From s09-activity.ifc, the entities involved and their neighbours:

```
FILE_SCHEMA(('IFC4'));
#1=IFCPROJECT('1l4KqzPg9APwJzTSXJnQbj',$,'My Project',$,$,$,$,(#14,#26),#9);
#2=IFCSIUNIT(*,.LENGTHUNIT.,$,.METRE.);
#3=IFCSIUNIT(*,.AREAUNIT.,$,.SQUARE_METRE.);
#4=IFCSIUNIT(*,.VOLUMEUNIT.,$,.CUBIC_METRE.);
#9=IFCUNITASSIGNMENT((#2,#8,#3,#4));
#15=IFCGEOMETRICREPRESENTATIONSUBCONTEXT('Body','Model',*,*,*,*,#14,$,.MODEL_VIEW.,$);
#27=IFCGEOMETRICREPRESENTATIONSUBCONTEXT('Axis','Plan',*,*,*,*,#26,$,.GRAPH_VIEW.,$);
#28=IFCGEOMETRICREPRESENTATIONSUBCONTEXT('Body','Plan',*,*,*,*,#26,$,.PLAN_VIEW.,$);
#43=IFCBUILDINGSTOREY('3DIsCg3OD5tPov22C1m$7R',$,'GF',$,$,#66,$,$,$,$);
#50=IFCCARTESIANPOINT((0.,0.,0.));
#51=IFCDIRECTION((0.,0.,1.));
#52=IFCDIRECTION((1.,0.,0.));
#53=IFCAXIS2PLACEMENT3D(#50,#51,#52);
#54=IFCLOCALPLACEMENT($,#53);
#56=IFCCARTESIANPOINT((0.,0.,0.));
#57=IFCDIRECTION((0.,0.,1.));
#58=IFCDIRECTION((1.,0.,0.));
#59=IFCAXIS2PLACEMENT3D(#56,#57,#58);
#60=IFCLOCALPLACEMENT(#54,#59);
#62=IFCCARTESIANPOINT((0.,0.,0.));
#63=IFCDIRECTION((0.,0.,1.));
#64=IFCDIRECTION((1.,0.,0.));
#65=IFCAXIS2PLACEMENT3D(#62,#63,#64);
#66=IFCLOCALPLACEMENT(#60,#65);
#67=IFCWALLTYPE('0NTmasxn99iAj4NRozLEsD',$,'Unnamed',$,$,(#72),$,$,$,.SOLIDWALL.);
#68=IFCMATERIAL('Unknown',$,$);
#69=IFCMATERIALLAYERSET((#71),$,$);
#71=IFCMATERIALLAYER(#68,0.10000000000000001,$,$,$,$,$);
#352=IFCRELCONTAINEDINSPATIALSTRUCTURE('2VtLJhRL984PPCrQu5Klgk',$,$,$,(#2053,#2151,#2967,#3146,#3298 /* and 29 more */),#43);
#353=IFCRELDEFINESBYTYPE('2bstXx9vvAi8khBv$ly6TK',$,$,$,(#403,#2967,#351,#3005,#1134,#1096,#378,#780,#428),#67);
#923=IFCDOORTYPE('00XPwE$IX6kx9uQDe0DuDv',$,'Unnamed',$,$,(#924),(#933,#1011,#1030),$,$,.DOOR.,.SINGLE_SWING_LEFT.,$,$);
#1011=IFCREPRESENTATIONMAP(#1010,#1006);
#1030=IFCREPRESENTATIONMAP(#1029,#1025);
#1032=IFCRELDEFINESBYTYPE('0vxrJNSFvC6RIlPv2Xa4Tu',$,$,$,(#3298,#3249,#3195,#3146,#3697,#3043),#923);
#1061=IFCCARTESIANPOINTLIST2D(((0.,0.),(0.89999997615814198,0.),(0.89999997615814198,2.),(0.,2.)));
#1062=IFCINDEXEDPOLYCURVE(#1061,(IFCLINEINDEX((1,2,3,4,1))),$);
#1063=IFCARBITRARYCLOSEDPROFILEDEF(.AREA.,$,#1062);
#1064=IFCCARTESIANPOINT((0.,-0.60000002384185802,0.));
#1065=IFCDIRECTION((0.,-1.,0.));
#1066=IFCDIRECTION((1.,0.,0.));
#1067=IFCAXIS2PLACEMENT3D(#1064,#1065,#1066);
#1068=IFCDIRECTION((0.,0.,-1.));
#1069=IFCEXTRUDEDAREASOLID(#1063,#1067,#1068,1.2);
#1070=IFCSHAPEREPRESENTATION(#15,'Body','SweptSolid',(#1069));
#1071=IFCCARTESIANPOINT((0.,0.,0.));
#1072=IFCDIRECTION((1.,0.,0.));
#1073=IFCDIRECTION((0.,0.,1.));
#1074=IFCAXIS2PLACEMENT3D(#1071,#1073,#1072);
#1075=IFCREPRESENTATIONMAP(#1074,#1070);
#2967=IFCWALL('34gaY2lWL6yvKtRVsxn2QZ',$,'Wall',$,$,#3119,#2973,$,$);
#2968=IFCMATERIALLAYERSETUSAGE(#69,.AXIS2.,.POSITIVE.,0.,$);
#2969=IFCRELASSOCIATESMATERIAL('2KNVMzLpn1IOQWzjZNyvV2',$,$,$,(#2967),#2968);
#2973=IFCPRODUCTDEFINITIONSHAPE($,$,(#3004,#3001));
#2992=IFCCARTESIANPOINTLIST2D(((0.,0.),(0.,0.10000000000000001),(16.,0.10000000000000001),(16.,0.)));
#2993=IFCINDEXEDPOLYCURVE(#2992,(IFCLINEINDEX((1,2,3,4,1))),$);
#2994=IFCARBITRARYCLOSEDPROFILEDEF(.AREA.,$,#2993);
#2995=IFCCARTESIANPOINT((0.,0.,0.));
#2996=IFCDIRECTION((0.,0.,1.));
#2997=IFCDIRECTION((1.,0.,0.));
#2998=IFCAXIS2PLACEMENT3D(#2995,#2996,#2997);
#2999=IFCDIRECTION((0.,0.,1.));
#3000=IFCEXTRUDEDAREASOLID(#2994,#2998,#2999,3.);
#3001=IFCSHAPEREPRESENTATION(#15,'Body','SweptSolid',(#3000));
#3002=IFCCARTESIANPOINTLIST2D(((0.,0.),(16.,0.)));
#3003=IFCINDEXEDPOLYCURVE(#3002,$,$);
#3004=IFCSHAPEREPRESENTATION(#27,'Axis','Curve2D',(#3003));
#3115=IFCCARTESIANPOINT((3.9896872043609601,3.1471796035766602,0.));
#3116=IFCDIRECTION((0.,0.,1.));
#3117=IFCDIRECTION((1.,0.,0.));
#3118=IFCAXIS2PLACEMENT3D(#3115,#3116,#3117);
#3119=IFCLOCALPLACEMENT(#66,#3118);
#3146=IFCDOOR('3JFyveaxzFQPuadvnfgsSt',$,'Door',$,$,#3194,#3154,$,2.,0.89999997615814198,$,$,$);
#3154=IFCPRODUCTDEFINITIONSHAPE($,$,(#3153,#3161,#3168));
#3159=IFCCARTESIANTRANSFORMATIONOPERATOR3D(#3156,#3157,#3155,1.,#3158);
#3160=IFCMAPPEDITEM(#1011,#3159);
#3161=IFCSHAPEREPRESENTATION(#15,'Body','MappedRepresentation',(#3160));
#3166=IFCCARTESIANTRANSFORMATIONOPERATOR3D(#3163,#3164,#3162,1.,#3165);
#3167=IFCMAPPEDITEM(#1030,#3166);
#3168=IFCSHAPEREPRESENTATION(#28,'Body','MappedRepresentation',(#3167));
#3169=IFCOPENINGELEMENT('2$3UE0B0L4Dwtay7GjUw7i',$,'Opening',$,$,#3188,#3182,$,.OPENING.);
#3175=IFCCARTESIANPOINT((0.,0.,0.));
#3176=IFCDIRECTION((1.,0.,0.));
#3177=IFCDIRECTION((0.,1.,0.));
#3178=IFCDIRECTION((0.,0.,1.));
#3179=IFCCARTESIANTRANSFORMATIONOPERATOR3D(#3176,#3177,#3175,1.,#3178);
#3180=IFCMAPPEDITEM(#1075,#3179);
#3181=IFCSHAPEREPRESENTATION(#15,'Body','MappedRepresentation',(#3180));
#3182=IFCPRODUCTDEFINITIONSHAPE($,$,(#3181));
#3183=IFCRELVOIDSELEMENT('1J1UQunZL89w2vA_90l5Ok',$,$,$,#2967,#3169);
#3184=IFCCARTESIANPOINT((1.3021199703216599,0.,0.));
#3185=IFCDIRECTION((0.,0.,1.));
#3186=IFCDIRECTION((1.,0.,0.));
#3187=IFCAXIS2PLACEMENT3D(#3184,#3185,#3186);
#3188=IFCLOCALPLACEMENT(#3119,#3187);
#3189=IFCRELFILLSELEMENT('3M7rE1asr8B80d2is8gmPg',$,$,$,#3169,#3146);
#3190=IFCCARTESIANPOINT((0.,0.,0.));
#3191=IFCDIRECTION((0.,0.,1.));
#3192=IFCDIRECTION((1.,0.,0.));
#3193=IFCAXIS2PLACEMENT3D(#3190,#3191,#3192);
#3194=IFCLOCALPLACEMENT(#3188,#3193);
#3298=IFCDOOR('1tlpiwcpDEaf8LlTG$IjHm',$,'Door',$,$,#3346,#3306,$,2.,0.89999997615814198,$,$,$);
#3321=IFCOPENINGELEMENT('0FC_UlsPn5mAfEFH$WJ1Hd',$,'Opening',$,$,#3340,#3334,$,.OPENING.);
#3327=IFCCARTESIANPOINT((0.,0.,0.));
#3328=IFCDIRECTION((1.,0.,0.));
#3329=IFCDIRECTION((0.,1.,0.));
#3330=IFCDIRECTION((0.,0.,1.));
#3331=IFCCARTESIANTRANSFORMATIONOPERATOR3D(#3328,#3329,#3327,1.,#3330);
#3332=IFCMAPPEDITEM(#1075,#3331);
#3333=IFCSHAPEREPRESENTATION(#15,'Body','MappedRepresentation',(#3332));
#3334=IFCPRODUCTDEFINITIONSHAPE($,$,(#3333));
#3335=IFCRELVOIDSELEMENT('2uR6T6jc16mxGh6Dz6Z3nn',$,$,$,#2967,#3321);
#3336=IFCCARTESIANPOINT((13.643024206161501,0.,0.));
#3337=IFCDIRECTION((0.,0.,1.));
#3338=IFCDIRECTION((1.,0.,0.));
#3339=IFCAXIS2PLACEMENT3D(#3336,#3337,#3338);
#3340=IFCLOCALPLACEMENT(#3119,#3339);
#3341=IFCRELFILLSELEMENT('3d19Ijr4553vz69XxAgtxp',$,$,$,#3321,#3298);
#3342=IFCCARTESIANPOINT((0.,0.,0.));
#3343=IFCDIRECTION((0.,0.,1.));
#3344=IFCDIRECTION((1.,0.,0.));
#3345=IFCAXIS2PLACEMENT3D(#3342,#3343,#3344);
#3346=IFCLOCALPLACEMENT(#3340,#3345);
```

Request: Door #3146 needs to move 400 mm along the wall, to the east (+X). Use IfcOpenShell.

```python
import ifcopenshell
import ifcopenshell.api.geometry
import ifcopenshell.util.placement
import ifcopenshell.util.unit

model = ifcopenshell.open("s09-activity.ifc")
unit_scale = ifcopenshell.util.unit.calculate_unit_scale(model)

door = model.by_id(3146)
opening = door.FillsVoids[0].RelatingOpeningElement
wall = opening.VoidsElements[0].RelatingBuildingElement

wall_matrix = ifcopenshell.util.placement.get_local_placement(wall.ObjectPlacement)
shift = wall_matrix[:3, 0] * 0.4 / unit_scale
before = ifcopenshell.util.placement.get_local_placement(door.ObjectPlacement)[:3, 3].copy()

# The door is placed relative to its opening, so it follows when the opening moves.
matrix = ifcopenshell.util.placement.get_local_placement(opening.ObjectPlacement)
matrix[:3, 3] += shift
ifcopenshell.api.geometry.edit_object_placement(
    model, product=opening, matrix=matrix, is_si=False, should_transform_children=True
)

after = ifcopenshell.util.placement.get_local_placement(door.ObjectPlacement)[:3, 3]
print("door moved by", (after - before).round(3) + 0.0)

model.write("s09-activity_rev.ifc")
```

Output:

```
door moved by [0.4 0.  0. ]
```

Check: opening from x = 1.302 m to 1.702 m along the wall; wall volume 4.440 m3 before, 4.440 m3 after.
